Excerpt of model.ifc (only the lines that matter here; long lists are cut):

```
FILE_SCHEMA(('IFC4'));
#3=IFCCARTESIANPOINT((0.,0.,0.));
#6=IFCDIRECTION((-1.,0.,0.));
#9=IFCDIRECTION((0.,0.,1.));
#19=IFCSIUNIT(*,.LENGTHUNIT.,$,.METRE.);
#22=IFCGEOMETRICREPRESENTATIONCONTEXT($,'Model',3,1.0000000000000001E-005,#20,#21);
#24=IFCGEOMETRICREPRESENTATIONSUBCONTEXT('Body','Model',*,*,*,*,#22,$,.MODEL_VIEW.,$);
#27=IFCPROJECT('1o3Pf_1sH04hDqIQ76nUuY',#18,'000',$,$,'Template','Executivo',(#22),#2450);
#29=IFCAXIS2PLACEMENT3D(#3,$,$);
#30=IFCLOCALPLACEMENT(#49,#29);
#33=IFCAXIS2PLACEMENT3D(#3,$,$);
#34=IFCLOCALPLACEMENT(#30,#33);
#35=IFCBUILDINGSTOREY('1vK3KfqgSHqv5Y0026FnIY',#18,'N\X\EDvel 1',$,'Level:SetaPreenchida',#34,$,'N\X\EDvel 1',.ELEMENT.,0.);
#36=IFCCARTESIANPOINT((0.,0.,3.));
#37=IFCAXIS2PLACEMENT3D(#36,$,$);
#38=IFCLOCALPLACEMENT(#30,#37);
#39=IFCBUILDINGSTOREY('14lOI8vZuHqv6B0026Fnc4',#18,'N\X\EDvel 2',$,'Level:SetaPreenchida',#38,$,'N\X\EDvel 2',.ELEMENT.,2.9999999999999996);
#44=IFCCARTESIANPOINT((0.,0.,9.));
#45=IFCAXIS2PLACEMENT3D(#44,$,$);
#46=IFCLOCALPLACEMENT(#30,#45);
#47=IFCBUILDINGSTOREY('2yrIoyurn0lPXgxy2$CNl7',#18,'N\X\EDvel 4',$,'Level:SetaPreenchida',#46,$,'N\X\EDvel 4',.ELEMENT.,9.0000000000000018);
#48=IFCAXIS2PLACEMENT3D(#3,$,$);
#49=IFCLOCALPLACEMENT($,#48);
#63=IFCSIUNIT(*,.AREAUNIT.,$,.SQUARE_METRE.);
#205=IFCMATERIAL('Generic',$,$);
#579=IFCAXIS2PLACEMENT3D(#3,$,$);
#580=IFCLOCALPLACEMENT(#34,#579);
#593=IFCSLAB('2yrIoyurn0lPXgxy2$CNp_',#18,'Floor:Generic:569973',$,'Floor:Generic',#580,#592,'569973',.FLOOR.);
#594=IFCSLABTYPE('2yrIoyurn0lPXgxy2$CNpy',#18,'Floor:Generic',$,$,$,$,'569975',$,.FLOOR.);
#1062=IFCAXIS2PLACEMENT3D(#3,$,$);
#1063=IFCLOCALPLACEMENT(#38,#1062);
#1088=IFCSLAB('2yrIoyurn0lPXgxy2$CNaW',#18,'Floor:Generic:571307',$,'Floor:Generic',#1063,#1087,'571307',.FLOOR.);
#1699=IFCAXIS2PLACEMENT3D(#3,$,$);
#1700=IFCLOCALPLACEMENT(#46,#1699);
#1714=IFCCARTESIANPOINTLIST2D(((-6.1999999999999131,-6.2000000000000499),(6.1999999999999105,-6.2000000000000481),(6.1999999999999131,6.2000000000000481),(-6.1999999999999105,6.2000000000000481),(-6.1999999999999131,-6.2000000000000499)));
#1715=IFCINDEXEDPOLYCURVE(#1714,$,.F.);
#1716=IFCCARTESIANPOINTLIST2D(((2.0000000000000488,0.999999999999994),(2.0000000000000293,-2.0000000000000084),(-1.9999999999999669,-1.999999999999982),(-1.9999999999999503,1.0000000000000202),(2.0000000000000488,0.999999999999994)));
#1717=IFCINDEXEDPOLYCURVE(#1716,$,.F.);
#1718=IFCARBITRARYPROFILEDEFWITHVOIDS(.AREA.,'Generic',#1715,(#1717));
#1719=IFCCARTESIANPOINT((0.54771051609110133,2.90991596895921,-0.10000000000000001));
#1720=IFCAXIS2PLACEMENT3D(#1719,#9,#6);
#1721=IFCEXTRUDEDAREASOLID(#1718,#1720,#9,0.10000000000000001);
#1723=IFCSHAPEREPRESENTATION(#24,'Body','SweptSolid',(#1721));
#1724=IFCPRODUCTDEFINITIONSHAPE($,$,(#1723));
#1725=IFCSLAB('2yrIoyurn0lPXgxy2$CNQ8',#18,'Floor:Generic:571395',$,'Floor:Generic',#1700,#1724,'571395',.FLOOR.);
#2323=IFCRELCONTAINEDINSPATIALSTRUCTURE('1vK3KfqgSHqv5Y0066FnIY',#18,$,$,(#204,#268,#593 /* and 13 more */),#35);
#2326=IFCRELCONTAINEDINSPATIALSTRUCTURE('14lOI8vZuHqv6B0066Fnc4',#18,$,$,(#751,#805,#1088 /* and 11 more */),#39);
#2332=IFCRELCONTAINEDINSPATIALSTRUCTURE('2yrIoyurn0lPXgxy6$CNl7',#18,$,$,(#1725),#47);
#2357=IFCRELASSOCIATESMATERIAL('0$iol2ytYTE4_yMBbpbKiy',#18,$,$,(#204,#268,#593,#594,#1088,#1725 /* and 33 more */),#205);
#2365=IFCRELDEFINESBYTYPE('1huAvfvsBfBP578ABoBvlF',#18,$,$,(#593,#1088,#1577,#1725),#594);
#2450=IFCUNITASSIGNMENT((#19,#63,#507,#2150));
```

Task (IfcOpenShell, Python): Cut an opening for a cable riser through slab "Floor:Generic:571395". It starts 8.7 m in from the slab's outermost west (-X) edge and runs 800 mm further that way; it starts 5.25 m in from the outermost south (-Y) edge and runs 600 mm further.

```python
import numpy as np
import ifcopenshell
import ifcopenshell.api.feature
import ifcopenshell.api.geometry
import ifcopenshell.api.root
import ifcopenshell.geom
import ifcopenshell.util.placement
import ifcopenshell.util.representation
import ifcopenshell.util.shape
import ifcopenshell.util.unit

model = ifcopenshell.open("model.ifc")
unit_scale = ifcopenshell.util.unit.calculate_unit_scale(model)
settings = ifcopenshell.geom.settings()


def volume(element):
    """Net volume in cubic metres, openings subtracted."""
    shape = ifcopenshell.geom.create_shape(settings, element)
    return ifcopenshell.util.shape.get_volume(shape.geometry)


slab = model.by_guid("2yrIoyurn0lPXgxy2$CNQ8")
before = volume(slab)

# Extent in the slab's own axes, in metres. The edges named are its -X and -Y sides.
slab_shape = ifcopenshell.geom.create_shape(settings, slab)
vertices = ifcopenshell.util.shape.get_vertices(slab_shape.geometry)
x_min, y_min, bottom = vertices.min(axis=0)
top = vertices[:, 2].max()

opening = ifcopenshell.api.root.create_entity(model, ifc_class="IfcOpeningElement", name="Cable riser opening", predefined_type="OPENING")
context = ifcopenshell.util.representation.get_context(model, "Model", "Body", "MODEL_VIEW")
width, depth = 0.8, 0.6
outline = [(0.0, 0.0), (width, 0.0), (width, depth), (0.0, depth), (0.0, 0.0)]
# Overshoot both faces by 50 mm so the cut is clean.
shape = ifcopenshell.api.geometry.add_slab_representation(
    model, context=context, depth=top - bottom + 0.1, polyline=outline
)
ifcopenshell.api.geometry.assign_representation(model, product=opening, representation=shape)

matrix = ifcopenshell.util.placement.get_local_placement(slab.ObjectPlacement)
matrix[:, 3] = matrix @ np.append(np.array([x_min + 8.7, y_min + 5.25, bottom - 0.05]) / unit_scale, 1.0)
ifcopenshell.api.geometry.edit_object_placement(model, product=opening, matrix=matrix, is_si=False)
ifcopenshell.api.feature.add_feature(model, feature=opening, element=slab)

after = volume(slab)

print(f"slab volume {before:.3f} -> {after:.3f} m3")

model.write("model_v2.ifc")
```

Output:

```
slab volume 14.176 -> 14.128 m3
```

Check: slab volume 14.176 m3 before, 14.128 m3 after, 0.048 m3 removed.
